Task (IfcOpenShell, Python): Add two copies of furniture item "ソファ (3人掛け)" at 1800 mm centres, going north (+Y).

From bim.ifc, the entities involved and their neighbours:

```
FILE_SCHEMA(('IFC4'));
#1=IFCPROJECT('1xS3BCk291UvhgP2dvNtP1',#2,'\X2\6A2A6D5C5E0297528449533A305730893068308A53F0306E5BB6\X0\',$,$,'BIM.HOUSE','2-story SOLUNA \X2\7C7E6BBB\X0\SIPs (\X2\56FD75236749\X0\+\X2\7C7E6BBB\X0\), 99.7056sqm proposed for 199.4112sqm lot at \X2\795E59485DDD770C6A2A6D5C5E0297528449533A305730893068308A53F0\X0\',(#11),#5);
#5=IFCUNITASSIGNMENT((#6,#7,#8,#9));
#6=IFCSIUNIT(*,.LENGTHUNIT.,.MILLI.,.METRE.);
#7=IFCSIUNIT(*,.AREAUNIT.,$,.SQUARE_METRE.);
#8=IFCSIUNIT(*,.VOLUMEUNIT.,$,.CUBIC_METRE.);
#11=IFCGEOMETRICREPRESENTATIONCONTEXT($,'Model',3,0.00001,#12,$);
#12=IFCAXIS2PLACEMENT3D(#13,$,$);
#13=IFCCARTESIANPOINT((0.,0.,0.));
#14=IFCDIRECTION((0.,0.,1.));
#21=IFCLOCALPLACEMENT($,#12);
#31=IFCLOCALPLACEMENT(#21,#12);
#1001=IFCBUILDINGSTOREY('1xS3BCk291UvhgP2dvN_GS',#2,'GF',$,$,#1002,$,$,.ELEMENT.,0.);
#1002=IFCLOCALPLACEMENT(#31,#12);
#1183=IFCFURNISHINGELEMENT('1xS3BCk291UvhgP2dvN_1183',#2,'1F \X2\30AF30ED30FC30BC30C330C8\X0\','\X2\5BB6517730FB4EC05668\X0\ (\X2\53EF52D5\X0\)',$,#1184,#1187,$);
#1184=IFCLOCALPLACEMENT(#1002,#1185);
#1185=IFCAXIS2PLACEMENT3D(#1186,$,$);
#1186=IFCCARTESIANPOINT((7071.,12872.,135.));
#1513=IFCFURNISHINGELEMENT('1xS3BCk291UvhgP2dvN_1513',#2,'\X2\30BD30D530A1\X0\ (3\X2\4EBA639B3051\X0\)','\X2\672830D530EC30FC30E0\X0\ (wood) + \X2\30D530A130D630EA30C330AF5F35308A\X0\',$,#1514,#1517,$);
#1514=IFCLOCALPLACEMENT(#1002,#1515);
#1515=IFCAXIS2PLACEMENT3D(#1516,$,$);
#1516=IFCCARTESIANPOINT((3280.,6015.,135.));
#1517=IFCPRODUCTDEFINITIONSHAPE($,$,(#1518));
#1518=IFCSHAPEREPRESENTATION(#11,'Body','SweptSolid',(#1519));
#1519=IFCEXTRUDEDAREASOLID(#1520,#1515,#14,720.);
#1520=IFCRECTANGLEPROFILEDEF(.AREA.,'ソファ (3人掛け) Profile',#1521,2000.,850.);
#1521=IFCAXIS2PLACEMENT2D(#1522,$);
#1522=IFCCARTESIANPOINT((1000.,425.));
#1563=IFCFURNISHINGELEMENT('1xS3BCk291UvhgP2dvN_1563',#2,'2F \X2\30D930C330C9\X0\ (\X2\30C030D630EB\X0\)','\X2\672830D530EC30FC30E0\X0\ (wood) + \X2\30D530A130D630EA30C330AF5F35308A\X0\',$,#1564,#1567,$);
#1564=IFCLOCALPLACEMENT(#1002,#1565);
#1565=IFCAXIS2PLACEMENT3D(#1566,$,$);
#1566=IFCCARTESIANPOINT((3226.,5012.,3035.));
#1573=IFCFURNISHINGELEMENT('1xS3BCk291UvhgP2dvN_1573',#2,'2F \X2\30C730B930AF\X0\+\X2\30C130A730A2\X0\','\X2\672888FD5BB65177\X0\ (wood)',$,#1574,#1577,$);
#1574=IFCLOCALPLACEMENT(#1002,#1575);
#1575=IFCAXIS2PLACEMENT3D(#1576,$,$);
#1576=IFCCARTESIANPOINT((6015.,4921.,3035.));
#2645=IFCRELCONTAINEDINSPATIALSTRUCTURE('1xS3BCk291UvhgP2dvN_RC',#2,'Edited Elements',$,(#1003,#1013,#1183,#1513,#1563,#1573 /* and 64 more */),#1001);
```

```python
import numpy as np
import ifcopenshell
import ifcopenshell.api.geometry
import ifcopenshell.api.root
import ifcopenshell.util.element
import ifcopenshell.util.placement

model = ifcopenshell.open("bim.ifc")


def reuse_history(source, copy):
    """copy_class also copies each property set's owner history, people and application; keep the originals."""
    for rel in copy.IsDefinedBy:
        if rel.is_a("IfcRelDefinesByProperties") and (history := rel.RelatingPropertyDefinition.OwnerHistory):
            rel.RelatingPropertyDefinition.OwnerHistory = source.OwnerHistory
            ifcopenshell.util.element.remove_deep2(model, history)


source = model.by_guid("1xS3BCk291UvhgP2dvN_1513")
base = ifcopenshell.util.placement.get_local_placement(source.ObjectPlacement)
step = np.array([0.0, 1.0, 0.0]) * 1800.0

for i in range(1, 3):
    copy = ifcopenshell.api.root.copy_class(model, product=source)
    copy.Representation = ifcopenshell.util.element.copy_deep(
        model, source.Representation, exclude=["IfcGeometricRepresentationContext", "IfcRepresentationMap"]
    )
    reuse_history(source, copy)
    matrix = base.copy()
    matrix[:3, 3] += i * step
    print("added at", matrix[:3, 3].round(3) + 0.0)
    ifcopenshell.api.geometry.edit_object_placement(model, product=copy, matrix=matrix, is_si=False)

model.write("bim_v2.ifc")
```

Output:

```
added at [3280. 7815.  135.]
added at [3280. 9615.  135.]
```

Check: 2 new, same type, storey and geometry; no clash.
